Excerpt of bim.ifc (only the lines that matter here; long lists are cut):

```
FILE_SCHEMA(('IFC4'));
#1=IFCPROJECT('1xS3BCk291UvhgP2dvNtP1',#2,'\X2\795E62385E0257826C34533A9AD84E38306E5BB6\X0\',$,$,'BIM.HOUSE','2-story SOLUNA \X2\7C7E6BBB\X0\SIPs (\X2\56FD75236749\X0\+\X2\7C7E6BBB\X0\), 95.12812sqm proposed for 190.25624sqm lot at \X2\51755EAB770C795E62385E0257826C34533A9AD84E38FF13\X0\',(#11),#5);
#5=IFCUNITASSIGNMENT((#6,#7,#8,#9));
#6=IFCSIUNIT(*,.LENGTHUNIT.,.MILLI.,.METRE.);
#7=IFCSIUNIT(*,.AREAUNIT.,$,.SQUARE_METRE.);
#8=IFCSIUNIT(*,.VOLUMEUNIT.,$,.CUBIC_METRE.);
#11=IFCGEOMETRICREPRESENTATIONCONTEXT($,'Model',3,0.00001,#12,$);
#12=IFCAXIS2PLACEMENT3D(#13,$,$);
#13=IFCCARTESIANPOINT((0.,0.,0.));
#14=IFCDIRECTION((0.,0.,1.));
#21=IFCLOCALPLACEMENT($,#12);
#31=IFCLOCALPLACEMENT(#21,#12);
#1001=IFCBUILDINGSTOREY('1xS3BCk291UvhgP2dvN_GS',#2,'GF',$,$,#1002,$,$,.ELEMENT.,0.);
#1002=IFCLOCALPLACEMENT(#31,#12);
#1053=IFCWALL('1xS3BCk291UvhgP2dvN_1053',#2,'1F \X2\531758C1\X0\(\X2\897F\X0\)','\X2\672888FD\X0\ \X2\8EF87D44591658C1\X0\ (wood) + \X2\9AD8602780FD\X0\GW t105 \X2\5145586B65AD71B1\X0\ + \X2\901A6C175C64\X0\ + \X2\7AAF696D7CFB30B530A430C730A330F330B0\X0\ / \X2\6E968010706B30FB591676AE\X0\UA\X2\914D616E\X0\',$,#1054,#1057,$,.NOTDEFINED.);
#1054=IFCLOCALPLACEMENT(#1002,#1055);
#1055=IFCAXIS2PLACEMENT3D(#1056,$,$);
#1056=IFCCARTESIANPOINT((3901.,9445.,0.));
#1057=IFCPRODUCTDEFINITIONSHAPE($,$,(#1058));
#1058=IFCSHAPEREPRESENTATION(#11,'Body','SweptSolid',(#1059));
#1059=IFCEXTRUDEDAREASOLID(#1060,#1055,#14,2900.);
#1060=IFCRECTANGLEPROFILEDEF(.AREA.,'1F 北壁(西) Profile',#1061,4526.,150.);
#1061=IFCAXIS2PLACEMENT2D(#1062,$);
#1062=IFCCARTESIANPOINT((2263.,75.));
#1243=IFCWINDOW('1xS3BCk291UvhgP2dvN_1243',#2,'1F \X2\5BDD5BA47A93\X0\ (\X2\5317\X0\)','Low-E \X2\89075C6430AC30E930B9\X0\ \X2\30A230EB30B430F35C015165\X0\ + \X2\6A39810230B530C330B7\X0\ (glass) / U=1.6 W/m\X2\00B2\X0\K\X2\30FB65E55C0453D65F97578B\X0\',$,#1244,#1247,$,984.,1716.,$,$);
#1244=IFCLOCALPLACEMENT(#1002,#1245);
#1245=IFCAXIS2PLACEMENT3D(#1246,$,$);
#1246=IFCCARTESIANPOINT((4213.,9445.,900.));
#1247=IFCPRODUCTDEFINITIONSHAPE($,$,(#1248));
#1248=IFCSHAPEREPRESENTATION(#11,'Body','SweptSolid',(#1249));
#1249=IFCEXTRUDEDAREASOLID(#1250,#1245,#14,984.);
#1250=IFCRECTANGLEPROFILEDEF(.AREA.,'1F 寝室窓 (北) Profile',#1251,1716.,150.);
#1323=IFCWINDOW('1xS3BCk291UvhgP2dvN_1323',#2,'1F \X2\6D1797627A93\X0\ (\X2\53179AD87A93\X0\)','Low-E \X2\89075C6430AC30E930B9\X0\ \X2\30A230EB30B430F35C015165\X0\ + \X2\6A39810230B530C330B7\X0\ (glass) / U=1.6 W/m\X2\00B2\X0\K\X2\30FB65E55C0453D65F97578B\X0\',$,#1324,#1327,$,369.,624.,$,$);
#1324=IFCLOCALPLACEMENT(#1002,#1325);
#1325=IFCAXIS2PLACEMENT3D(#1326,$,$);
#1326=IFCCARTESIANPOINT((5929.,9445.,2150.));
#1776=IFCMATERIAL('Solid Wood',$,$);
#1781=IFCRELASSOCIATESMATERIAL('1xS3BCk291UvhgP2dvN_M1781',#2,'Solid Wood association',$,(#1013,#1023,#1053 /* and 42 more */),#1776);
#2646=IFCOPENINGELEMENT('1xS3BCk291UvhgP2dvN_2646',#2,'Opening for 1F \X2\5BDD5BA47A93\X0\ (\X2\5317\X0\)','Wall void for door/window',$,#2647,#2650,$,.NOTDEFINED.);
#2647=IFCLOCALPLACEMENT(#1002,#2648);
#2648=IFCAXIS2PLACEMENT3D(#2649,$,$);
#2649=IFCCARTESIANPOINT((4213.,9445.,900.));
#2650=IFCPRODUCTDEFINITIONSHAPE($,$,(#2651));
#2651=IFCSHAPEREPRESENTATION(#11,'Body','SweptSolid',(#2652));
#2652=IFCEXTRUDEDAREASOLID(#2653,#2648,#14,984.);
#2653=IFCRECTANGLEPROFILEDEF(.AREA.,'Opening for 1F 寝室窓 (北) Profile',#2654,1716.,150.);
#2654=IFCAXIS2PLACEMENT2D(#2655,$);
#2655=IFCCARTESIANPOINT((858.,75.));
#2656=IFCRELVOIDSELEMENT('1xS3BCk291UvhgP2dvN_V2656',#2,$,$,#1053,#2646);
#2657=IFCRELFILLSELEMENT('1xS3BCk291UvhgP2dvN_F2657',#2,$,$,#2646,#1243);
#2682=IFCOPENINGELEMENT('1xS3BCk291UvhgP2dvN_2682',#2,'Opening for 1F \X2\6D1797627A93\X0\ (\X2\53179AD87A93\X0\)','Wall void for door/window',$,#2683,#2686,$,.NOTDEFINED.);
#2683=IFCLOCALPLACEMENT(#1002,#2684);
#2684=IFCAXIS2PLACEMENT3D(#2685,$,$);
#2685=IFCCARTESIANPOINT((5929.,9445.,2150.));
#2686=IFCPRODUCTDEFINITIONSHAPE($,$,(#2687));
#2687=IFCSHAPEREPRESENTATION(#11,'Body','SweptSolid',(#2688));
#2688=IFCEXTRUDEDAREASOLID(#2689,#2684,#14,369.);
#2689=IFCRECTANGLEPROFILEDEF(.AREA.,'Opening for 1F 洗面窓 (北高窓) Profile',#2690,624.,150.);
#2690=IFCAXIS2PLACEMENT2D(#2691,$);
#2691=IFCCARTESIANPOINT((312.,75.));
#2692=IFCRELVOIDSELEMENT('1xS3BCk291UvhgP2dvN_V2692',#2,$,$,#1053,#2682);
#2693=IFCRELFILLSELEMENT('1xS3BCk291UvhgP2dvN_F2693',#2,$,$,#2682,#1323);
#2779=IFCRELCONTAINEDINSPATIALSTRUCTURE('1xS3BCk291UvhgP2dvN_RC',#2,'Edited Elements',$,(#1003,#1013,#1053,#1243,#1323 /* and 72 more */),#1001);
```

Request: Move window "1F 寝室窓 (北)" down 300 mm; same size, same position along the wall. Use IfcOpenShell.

```python
import numpy as np
import ifcopenshell
import ifcopenshell.api.geometry
import ifcopenshell.util.placement
import ifcopenshell.util.unit

model = ifcopenshell.open("bim.ifc")
unit_scale = ifcopenshell.util.unit.calculate_unit_scale(model)

window = model.by_guid("1xS3BCk291UvhgP2dvN_1243")
opening = window.FillsVoids[0].RelatingOpeningElement
dz = -0.3 / unit_scale

shift = np.array([0.0, 0.0, dz])
# The window is not placed relative to its opening, so move both.
for product in (opening, window):
    matrix = ifcopenshell.util.placement.get_local_placement(product.ObjectPlacement)
    matrix[:3, 3] += shift
    ifcopenshell.api.geometry.edit_object_placement(model, product=product, matrix=matrix, is_si=False)

print(f"moved by {dz * unit_scale:+.3f} m")

model.write("bim-out.ifc")
```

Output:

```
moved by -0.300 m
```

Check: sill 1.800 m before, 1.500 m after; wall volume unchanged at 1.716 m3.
